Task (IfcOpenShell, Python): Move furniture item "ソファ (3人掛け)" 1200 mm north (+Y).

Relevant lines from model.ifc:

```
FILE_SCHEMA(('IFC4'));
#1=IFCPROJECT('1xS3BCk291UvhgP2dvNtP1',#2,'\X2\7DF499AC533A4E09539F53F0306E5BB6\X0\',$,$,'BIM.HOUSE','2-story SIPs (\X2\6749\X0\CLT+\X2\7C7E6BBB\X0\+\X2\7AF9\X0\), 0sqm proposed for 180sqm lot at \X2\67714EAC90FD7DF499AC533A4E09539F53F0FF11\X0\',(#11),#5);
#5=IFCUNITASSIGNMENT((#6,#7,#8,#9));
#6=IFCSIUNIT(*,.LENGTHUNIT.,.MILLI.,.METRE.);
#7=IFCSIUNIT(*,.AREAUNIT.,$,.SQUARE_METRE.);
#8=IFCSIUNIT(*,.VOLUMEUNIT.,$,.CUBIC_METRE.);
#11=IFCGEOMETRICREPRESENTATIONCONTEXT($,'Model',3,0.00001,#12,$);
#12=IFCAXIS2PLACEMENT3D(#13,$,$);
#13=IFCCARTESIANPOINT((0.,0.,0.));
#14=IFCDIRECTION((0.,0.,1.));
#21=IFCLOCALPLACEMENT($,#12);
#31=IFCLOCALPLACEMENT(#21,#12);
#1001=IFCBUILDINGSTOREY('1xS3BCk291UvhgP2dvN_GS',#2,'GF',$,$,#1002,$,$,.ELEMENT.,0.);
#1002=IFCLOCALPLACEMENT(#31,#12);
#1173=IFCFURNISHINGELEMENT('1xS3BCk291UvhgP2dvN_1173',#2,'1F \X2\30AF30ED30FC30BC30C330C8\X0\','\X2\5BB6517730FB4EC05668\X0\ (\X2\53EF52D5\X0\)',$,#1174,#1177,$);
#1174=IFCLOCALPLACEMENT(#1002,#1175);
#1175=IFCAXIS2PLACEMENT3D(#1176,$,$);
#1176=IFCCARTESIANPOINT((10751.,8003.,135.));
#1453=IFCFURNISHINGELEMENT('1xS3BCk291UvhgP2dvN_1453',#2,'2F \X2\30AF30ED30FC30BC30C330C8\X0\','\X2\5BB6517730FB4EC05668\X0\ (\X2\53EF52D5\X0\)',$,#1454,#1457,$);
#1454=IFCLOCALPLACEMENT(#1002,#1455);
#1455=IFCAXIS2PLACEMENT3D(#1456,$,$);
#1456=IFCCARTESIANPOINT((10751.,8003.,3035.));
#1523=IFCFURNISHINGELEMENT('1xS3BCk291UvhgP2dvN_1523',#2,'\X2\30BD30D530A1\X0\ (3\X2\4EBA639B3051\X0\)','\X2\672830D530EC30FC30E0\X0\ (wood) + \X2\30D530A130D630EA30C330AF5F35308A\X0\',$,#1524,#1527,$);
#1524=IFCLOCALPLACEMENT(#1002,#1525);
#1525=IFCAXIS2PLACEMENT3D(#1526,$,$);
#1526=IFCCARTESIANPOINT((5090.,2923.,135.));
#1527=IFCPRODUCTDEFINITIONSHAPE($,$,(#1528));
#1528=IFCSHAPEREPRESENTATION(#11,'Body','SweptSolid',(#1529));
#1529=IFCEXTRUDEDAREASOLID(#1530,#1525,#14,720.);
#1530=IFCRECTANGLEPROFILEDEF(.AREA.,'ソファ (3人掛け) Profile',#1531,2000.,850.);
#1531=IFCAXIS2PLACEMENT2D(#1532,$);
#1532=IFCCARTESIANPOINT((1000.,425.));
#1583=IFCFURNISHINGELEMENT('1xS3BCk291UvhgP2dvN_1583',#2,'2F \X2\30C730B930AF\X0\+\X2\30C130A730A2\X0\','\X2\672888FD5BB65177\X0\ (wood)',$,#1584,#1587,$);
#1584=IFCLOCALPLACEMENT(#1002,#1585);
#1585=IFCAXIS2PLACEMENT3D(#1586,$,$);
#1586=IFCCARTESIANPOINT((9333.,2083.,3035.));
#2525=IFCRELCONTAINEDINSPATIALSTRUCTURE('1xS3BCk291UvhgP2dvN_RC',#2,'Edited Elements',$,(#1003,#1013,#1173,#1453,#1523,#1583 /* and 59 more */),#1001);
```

```python
import ifcopenshell
import ifcopenshell.api.geometry
import ifcopenshell.util.placement
import ifcopenshell.util.unit

model = ifcopenshell.open("model.ifc")
unit_scale = ifcopenshell.util.unit.calculate_unit_scale(model)

item = model.by_guid("1xS3BCk291UvhgP2dvN_1523")
matrix = ifcopenshell.util.placement.get_local_placement(item.ObjectPlacement)
matrix[1, 3] += 1.2 / unit_scale
ifcopenshell.api.geometry.edit_object_placement(model, product=item, matrix=matrix, is_si=False)

print(ifcopenshell.util.placement.get_local_placement(item.ObjectPlacement).round(3) + 0.0)

model.write("model_edited.ifc")
```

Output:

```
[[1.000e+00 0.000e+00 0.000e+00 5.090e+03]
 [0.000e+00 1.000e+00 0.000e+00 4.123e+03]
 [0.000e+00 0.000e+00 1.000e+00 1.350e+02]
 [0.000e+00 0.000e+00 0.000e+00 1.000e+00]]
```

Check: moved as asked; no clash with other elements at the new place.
